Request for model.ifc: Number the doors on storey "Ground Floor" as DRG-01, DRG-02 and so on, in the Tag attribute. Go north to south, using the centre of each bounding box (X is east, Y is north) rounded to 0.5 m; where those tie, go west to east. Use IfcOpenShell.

First a look at what the model holds.

```python
import ifcopenshell
import ifcopenshell.util.element
import ifcopenshell.util.placement

model = ifcopenshell.open("model.ifc")
print(model.schema)
storey = next(s for s in model.by_type("IfcBuildingStorey") if s.Name == "Ground Floor")
doors = [e for e in ifcopenshell.util.element.get_decomposition(storey) if e.is_a("IfcDoor")]
for e in sorted(doors, key=lambda e: e.id()):
    origin = ifcopenshell.util.placement.get_local_placement(e.ObjectPlacement)[:3, 3]
    print(e.id(), e.Tag, e.Name, origin.round(2) + 0.0, sep=" | ")
```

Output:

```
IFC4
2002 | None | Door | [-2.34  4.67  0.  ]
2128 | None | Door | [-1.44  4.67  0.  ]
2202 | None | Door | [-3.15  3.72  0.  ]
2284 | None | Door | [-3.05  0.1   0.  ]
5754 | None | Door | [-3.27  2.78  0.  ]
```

```python
import ifcopenshell
import ifcopenshell.geom
import ifcopenshell.util.element
import ifcopenshell.util.shape

model = ifcopenshell.open("model.ifc")
settings = ifcopenshell.geom.settings()
settings.set("use-world-coords", True)


def centre(element):
    shape = ifcopenshell.geom.create_shape(settings, element)
    return ifcopenshell.util.shape.get_bbox_centroid(shape.geometry)


storey = next(s for s in model.by_type("IfcBuildingStorey") if s.Name == "Ground Floor")
doors = [e for e in ifcopenshell.util.element.get_decomposition(storey) if e.is_a("IfcDoor")]

# Insertion points can sit at a corner or the storey origin, so sort by the geometry (in metres).
centres = {e: centre(e) for e in doors}
doors.sort(key=lambda e: (-round(centres[e][1] / 0.5), centres[e][0]))

for i, e in enumerate(doors, start=1):
    number = f"DRG-{i:02d}"
    e.Tag = number
    print(e.id(), number)

model.write("model-out.ifc")
```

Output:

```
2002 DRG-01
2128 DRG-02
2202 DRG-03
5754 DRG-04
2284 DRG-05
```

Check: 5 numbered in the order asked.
